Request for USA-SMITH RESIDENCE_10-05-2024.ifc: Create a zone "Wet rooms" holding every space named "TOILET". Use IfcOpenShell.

First a look at what the model holds.

```python
import ifcopenshell

model = ifcopenshell.open("USA-SMITH RESIDENCE_10-05-2024.ifc")
print(model.schema)
seen = {}
for space in model.by_type("IfcSpace"):
    seen[space.LongName] = seen.get(space.LongName, 0) + 1
for name, count in sorted(seen.items(), key=str):
    print(count, "x", name)
print("zones:", [z.Name for z in model.by_type("IfcZone")][:20])
```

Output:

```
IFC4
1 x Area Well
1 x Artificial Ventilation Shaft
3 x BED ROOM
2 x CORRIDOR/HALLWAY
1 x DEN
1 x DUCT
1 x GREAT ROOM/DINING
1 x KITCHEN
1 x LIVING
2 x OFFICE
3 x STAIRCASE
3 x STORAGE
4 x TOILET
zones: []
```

```python
import ifcopenshell
import ifcopenshell.api.group
import ifcopenshell.api.root

model = ifcopenshell.open("USA-SMITH RESIDENCE_10-05-2024.ifc")

names = {"TOILET"}
spaces = [s for s in model.by_type("IfcSpace") if s.LongName in names]

zone = ifcopenshell.api.root.create_entity(model, ifc_class="IfcZone", name="Wet rooms")
ifcopenshell.api.group.assign_group(model, products=spaces, group=zone)
print(len(spaces), "spaces in", zone.Name)

model.write("USA-SMITH RESIDENCE_10-05-2024_updated.ifc")
```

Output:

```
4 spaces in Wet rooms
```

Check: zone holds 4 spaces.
